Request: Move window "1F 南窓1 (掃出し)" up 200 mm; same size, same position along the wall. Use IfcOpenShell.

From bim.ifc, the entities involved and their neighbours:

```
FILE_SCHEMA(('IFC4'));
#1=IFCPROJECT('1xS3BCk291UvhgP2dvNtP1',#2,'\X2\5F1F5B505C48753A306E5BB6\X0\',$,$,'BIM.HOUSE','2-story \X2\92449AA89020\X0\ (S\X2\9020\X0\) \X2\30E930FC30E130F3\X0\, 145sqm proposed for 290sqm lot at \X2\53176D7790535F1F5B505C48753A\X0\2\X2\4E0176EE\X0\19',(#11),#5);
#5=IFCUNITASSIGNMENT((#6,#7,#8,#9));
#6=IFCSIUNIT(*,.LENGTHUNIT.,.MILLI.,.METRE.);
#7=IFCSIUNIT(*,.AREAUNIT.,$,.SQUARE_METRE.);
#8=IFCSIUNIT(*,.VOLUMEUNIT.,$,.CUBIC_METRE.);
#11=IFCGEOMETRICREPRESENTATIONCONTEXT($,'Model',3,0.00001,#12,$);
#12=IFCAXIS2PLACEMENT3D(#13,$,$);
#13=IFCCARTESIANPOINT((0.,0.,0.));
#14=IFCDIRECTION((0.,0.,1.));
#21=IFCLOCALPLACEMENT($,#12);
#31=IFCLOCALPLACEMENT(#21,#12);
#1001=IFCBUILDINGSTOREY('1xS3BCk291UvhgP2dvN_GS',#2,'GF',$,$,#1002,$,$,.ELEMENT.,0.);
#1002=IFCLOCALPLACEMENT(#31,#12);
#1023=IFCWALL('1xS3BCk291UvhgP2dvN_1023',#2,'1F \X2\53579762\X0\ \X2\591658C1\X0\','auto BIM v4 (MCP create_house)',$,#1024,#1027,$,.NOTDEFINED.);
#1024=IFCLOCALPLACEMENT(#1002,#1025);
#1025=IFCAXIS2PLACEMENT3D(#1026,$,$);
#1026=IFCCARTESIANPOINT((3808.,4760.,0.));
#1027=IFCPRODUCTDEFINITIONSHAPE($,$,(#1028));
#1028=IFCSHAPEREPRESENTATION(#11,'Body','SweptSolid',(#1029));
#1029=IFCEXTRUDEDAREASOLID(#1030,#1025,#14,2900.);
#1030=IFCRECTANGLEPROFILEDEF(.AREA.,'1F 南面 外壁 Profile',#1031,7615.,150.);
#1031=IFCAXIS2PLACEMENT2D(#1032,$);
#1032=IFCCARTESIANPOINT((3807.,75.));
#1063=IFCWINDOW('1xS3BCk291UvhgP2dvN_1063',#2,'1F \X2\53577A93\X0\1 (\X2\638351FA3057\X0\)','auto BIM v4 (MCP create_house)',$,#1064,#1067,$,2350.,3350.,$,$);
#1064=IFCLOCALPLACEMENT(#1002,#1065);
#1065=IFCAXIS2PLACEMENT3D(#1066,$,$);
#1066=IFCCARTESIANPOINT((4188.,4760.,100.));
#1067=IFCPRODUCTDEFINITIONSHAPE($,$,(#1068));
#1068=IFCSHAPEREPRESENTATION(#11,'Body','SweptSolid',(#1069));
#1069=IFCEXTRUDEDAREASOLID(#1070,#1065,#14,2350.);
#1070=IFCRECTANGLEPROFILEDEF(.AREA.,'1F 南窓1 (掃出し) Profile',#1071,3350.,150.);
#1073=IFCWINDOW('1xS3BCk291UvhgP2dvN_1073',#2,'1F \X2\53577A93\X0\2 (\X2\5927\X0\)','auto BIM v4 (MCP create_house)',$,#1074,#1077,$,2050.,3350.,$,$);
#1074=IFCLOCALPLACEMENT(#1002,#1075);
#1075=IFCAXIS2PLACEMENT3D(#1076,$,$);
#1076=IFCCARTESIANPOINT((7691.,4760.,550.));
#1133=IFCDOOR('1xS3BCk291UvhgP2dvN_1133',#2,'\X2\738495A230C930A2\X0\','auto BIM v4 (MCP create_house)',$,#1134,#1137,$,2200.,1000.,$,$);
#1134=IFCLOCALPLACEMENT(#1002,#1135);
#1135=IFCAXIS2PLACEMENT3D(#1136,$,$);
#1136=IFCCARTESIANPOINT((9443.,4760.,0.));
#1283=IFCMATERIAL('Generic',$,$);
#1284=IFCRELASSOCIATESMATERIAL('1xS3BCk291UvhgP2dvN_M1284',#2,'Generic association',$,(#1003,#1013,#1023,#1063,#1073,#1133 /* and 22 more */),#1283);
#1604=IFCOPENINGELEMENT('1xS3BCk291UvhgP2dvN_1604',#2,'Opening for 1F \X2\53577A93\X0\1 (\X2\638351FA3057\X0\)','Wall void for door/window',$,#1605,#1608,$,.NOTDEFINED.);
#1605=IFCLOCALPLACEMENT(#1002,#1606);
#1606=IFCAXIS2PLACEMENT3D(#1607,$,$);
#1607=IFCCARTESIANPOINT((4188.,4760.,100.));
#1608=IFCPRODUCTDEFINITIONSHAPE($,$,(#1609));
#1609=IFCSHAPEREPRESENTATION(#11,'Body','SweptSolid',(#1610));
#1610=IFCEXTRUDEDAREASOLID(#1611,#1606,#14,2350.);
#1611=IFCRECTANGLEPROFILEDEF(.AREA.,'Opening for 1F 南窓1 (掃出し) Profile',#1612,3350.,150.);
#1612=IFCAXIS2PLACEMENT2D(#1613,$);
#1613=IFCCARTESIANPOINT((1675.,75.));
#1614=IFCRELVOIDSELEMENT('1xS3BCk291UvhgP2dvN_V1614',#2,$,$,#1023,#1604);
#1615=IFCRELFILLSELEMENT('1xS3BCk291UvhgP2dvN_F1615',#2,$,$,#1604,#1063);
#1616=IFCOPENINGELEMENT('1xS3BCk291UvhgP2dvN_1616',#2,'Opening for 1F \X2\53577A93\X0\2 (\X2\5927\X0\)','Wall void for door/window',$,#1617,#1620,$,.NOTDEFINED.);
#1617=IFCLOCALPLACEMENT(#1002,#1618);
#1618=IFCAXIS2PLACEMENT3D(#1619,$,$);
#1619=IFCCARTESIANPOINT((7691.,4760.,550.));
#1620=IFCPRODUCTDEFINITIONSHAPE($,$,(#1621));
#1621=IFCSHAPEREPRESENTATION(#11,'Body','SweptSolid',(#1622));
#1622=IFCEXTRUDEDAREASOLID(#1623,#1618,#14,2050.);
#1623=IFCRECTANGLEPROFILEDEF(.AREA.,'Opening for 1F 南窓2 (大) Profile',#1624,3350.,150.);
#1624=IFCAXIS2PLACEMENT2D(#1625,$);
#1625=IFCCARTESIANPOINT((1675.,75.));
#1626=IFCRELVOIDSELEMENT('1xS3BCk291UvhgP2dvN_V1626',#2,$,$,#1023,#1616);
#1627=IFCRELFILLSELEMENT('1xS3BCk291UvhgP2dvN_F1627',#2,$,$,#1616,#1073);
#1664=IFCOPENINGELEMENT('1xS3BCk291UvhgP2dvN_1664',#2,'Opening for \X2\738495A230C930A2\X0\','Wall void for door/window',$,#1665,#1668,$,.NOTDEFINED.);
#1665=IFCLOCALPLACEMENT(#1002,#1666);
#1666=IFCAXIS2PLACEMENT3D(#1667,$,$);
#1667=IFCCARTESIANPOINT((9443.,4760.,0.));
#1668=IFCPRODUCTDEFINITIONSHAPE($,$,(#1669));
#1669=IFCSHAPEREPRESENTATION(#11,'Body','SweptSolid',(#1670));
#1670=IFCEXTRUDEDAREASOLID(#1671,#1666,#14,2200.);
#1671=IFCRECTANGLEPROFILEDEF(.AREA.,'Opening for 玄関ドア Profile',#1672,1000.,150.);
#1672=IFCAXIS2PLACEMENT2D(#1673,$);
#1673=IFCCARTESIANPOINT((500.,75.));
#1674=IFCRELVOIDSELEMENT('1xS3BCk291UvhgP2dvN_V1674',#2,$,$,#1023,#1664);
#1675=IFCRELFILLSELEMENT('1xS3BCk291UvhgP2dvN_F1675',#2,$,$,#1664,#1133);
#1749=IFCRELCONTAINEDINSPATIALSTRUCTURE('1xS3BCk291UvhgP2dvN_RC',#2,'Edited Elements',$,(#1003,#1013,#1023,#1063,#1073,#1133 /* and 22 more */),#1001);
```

```python
import numpy as np
import ifcopenshell
import ifcopenshell.api.geometry
import ifcopenshell.util.placement
import ifcopenshell.util.unit

model = ifcopenshell.open("bim.ifc")
unit_scale = ifcopenshell.util.unit.calculate_unit_scale(model)

window = model.by_id(1063)
opening = window.FillsVoids[0].RelatingOpeningElement
dz = 200.0

shift = np.array([0.0, 0.0, dz])
# The window is not placed relative to its opening, so move both.
for product in (opening, window):
    matrix = ifcopenshell.util.placement.get_local_placement(product.ObjectPlacement)
    matrix[:3, 3] += shift
    ifcopenshell.api.geometry.edit_object_placement(model, product=product, matrix=matrix, is_si=False)

print(f"moved by {dz * unit_scale:+.3f} m")

model.write("bim_edited.ifc")
```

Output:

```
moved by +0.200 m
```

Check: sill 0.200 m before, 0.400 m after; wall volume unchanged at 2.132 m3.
